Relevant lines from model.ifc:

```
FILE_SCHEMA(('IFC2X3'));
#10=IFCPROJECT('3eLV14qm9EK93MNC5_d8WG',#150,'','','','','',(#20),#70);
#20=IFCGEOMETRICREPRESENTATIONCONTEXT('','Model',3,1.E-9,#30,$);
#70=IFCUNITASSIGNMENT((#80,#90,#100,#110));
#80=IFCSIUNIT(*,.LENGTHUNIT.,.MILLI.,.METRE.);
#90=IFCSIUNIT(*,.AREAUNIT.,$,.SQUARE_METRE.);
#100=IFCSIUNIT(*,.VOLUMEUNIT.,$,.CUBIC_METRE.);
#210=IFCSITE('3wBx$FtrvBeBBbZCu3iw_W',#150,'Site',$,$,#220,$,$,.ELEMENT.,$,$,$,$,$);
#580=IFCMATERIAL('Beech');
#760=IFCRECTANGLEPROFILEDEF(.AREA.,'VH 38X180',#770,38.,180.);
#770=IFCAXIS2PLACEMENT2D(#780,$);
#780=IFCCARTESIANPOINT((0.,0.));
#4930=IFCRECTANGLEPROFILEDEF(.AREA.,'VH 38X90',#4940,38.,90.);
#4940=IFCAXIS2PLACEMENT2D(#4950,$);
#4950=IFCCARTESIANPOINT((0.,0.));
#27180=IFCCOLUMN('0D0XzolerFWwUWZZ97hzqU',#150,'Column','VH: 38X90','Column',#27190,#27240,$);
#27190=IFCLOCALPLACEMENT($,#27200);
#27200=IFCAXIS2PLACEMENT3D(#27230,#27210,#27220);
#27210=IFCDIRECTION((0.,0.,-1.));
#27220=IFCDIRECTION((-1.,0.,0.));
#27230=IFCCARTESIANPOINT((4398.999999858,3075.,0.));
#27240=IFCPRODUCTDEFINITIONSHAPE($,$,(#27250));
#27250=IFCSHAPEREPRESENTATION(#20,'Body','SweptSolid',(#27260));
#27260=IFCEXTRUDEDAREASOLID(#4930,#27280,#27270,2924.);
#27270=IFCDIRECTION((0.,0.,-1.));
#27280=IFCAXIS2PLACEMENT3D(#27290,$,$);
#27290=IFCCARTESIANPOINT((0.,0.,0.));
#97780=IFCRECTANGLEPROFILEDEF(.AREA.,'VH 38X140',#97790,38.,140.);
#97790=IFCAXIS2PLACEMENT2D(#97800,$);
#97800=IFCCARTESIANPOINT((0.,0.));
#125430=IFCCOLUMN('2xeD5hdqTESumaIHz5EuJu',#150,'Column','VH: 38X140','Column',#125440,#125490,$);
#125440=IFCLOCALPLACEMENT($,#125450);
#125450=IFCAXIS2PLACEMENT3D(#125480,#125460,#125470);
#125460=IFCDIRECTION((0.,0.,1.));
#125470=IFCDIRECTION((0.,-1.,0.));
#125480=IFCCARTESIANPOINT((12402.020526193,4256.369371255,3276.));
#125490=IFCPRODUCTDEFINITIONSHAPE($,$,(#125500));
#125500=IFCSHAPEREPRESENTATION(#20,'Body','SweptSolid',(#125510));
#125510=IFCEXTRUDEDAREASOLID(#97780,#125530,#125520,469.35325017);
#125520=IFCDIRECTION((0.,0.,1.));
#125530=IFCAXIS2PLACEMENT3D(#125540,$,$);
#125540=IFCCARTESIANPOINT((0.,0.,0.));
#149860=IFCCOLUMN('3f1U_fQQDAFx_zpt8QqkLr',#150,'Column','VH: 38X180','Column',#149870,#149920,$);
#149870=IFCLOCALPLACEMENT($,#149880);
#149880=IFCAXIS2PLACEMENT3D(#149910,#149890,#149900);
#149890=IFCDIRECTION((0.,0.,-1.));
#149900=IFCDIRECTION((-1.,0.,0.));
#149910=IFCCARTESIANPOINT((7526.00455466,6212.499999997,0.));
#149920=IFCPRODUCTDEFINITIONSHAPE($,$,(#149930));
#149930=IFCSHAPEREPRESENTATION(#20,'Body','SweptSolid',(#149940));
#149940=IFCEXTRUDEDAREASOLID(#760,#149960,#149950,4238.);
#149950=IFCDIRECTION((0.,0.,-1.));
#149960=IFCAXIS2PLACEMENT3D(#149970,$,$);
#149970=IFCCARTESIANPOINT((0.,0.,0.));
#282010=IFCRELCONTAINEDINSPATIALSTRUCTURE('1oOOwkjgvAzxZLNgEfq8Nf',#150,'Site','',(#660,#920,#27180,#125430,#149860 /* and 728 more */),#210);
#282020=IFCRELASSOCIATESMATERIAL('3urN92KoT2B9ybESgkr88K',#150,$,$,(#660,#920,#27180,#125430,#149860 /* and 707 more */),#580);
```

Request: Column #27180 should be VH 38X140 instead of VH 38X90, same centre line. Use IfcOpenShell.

```python
import ifcopenshell
import ifcopenshell.util.element

model = ifcopenshell.open("model.ifc")

member = model.by_guid("0D0XzolerFWwUWZZ97hzqU")
source = next(p for p in model.by_type("IfcRectangleProfileDef") if p.ProfileName == "VH 38X140")

body = next(r for r in member.Representation.Representations if r.RepresentationIdentifier == "Body")
solid = body.Items[0]
old_profile = solid.SweptArea

# Copy the section's sizes but keep this member's own profile position.
profile = ifcopenshell.util.element.copy(model, source)
profile.Position = old_profile.Position
solid.SweptArea = profile
if not model.get_total_inverses(old_profile):
    ifcopenshell.util.element.remove_deep2(model, old_profile)

print(solid.SweptArea)

model.write("model_rev.ifc")
```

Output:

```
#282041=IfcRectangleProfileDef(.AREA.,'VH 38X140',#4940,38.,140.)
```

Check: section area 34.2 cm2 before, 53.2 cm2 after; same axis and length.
